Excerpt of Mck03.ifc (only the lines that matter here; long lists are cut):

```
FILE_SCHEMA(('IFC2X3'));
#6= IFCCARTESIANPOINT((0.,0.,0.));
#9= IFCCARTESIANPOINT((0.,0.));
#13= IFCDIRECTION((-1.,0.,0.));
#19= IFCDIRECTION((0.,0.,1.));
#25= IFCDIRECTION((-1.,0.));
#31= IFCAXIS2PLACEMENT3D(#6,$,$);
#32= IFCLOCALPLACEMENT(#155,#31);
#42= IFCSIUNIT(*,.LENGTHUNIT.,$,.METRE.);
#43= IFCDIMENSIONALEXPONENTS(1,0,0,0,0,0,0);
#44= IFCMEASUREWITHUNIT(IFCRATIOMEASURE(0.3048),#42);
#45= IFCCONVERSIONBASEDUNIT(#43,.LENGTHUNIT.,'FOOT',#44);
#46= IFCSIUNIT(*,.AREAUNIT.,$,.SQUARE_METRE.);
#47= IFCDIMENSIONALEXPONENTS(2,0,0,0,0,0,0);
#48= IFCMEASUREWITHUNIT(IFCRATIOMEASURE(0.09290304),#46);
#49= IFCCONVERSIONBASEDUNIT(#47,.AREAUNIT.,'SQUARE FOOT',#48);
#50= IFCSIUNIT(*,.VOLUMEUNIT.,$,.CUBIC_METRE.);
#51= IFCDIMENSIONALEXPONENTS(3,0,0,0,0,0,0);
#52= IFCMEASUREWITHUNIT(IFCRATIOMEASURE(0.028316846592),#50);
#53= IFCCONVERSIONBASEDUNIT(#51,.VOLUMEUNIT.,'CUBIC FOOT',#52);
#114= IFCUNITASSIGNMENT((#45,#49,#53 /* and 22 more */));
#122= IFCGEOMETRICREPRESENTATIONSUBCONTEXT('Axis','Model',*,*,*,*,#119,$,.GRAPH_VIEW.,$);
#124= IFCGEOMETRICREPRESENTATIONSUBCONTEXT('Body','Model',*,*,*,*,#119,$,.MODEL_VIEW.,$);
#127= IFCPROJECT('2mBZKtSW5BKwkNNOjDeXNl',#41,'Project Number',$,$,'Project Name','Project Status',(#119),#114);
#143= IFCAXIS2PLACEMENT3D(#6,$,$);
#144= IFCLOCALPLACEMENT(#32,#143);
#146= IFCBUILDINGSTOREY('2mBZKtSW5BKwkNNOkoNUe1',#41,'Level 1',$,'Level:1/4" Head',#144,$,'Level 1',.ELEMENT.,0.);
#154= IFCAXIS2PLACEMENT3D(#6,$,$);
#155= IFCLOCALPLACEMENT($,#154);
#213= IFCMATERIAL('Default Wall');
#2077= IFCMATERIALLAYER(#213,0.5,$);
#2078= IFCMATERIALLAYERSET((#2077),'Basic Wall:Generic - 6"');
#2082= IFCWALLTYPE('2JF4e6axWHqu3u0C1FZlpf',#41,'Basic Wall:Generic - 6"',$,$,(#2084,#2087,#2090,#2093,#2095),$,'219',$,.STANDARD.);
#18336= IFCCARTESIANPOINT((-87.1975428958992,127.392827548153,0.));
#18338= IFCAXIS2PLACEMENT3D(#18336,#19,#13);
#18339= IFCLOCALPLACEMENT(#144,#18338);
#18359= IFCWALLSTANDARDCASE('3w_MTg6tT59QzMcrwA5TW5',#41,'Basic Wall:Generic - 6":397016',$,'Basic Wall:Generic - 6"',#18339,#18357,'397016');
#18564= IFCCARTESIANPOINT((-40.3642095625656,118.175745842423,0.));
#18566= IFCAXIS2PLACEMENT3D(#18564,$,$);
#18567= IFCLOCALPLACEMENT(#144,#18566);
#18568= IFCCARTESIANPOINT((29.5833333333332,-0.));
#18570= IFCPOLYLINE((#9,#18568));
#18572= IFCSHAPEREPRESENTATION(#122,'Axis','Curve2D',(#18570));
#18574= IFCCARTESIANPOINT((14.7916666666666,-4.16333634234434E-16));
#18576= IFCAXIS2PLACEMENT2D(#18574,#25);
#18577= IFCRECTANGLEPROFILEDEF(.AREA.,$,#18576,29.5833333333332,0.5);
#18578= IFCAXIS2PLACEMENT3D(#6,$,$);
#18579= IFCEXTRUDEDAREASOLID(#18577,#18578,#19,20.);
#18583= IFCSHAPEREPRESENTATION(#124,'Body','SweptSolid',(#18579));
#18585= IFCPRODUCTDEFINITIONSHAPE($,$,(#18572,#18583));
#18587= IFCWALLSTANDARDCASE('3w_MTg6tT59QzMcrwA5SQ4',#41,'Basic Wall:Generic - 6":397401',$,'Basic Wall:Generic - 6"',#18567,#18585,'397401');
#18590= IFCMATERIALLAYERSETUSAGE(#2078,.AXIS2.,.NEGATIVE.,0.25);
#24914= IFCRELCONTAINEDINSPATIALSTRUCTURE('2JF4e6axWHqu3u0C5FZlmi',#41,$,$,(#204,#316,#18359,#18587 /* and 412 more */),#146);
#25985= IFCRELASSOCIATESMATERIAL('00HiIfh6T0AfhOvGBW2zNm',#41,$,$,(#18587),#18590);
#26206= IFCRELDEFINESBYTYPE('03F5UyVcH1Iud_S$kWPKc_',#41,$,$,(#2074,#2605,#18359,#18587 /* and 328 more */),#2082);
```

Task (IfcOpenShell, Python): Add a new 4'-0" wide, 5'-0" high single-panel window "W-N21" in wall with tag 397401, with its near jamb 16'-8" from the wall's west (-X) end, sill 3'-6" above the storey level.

```python
import numpy as np
import ifcopenshell
import ifcopenshell.api.feature
import ifcopenshell.api.geometry
import ifcopenshell.api.root
import ifcopenshell.api.spatial
import ifcopenshell.api.type
import ifcopenshell.geom
import ifcopenshell.util.element
import ifcopenshell.util.placement
import ifcopenshell.util.representation
import ifcopenshell.util.shape
import ifcopenshell.util.unit

model = ifcopenshell.open("Mck03.ifc")
unit_scale = ifcopenshell.util.unit.calculate_unit_scale(model)
settings = ifcopenshell.geom.settings()


def volume(element):
    """Net volume in cubic metres, openings subtracted."""
    shape = ifcopenshell.geom.create_shape(settings, element)
    return ifcopenshell.util.shape.get_volume(shape.geometry)


wall = model.by_guid("3w_MTg6tT59QzMcrwA5SQ4")
storey = ifcopenshell.util.element.get_container(wall, ifc_class="IfcBuildingStorey")
context = ifcopenshell.util.representation.get_context(model, "Model", "Body", "MODEL_VIEW")
before = volume(wall)

width, height, from_end, sill = 1.2192, 1.524, 5.08, 1.0668  # metres

# The wall runs along its own X axis, and the end named is its -X end.
wall_shape = ifcopenshell.geom.create_shape(settings, wall)
x, y, z = ifcopenshell.util.shape.get_vertices(wall_shape.geometry).T
start = x.min() + from_end
face, thickness = float(y.min()), float(y.max() - y.min())
wall_matrix = ifcopenshell.util.placement.get_local_placement(wall.ObjectPlacement)
level = ifcopenshell.util.placement.get_local_placement(storey.ObjectPlacement)[2, 3]


def in_wall(x, y):
    """Placement at x, y metres in the wall's axes, at sill height."""
    matrix = wall_matrix.copy()
    matrix[:, 3] = wall_matrix @ np.array([x / unit_scale, y / unit_scale, 0.0, 1.0])
    matrix[2, 3] = level + sill / unit_scale
    return matrix


# Opening: a box that overshoots both wall faces by 50 mm.
opening = ifcopenshell.api.root.create_entity(model, ifc_class="IfcOpeningElement")
box = ifcopenshell.api.geometry.add_wall_representation(
    model, context=context, length=width, height=height, thickness=thickness + 0.1
)
ifcopenshell.api.geometry.assign_representation(model, product=opening, representation=box)
ifcopenshell.api.geometry.edit_object_placement(model, product=opening, matrix=in_wall(start, face - 0.05), is_si=False)
ifcopenshell.api.feature.add_feature(model, feature=opening, element=wall)

window = ifcopenshell.api.root.create_entity(model, ifc_class="IfcWindow", name="W-N21")
window.OverallWidth, window.OverallHeight = width / unit_scale, height / unit_scale
body = ifcopenshell.api.geometry.add_window_representation(
    model,
    context=context,
    overall_width=window.OverallWidth,
    overall_height=window.OverallHeight,
    partition_type="SINGLE_PANEL",
)
ifcopenshell.api.geometry.assign_representation(model, product=window, representation=body)
ifcopenshell.api.spatial.assign_container(model, products=[window], relating_structure=storey)
fills = ifcopenshell.api.feature.add_filling(model, opening=opening, element=window)
fills.OwnerHistory = window.OwnerHistory  # required in IFC2X3

# IFC2X3 keeps the operation on the window style.
style = ifcopenshell.api.root.create_entity(model, ifc_class="IfcWindowStyle", name="W-N21")
style.OperationType, style.ConstructionType = "SINGLE_PANEL", "NOTDEFINED"
style.ParameterTakesPrecedence = style.Sizeable = False
ifcopenshell.api.type.assign_type(model, related_objects=[window], relating_type=style)

# Centre the window in the wall's thickness.
ifcopenshell.api.geometry.edit_object_placement(model, product=window, matrix=in_wall(start, face), is_si=False)
window_shape = ifcopenshell.geom.create_shape(settings, window)
depth = ifcopenshell.util.shape.get_vertices(window_shape.geometry)[:, 1]
offset = face + thickness / 2 - (depth.min() + depth.max()) / 2
ifcopenshell.api.geometry.edit_object_placement(model, product=window, matrix=in_wall(start, offset), is_si=False)

after = volume(wall)

print(f"wall volume {before:.3f} -> {after:.3f} m3")

model.write("Mck03_updated.ifc")
```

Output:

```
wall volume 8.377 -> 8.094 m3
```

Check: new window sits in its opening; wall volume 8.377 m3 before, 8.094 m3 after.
